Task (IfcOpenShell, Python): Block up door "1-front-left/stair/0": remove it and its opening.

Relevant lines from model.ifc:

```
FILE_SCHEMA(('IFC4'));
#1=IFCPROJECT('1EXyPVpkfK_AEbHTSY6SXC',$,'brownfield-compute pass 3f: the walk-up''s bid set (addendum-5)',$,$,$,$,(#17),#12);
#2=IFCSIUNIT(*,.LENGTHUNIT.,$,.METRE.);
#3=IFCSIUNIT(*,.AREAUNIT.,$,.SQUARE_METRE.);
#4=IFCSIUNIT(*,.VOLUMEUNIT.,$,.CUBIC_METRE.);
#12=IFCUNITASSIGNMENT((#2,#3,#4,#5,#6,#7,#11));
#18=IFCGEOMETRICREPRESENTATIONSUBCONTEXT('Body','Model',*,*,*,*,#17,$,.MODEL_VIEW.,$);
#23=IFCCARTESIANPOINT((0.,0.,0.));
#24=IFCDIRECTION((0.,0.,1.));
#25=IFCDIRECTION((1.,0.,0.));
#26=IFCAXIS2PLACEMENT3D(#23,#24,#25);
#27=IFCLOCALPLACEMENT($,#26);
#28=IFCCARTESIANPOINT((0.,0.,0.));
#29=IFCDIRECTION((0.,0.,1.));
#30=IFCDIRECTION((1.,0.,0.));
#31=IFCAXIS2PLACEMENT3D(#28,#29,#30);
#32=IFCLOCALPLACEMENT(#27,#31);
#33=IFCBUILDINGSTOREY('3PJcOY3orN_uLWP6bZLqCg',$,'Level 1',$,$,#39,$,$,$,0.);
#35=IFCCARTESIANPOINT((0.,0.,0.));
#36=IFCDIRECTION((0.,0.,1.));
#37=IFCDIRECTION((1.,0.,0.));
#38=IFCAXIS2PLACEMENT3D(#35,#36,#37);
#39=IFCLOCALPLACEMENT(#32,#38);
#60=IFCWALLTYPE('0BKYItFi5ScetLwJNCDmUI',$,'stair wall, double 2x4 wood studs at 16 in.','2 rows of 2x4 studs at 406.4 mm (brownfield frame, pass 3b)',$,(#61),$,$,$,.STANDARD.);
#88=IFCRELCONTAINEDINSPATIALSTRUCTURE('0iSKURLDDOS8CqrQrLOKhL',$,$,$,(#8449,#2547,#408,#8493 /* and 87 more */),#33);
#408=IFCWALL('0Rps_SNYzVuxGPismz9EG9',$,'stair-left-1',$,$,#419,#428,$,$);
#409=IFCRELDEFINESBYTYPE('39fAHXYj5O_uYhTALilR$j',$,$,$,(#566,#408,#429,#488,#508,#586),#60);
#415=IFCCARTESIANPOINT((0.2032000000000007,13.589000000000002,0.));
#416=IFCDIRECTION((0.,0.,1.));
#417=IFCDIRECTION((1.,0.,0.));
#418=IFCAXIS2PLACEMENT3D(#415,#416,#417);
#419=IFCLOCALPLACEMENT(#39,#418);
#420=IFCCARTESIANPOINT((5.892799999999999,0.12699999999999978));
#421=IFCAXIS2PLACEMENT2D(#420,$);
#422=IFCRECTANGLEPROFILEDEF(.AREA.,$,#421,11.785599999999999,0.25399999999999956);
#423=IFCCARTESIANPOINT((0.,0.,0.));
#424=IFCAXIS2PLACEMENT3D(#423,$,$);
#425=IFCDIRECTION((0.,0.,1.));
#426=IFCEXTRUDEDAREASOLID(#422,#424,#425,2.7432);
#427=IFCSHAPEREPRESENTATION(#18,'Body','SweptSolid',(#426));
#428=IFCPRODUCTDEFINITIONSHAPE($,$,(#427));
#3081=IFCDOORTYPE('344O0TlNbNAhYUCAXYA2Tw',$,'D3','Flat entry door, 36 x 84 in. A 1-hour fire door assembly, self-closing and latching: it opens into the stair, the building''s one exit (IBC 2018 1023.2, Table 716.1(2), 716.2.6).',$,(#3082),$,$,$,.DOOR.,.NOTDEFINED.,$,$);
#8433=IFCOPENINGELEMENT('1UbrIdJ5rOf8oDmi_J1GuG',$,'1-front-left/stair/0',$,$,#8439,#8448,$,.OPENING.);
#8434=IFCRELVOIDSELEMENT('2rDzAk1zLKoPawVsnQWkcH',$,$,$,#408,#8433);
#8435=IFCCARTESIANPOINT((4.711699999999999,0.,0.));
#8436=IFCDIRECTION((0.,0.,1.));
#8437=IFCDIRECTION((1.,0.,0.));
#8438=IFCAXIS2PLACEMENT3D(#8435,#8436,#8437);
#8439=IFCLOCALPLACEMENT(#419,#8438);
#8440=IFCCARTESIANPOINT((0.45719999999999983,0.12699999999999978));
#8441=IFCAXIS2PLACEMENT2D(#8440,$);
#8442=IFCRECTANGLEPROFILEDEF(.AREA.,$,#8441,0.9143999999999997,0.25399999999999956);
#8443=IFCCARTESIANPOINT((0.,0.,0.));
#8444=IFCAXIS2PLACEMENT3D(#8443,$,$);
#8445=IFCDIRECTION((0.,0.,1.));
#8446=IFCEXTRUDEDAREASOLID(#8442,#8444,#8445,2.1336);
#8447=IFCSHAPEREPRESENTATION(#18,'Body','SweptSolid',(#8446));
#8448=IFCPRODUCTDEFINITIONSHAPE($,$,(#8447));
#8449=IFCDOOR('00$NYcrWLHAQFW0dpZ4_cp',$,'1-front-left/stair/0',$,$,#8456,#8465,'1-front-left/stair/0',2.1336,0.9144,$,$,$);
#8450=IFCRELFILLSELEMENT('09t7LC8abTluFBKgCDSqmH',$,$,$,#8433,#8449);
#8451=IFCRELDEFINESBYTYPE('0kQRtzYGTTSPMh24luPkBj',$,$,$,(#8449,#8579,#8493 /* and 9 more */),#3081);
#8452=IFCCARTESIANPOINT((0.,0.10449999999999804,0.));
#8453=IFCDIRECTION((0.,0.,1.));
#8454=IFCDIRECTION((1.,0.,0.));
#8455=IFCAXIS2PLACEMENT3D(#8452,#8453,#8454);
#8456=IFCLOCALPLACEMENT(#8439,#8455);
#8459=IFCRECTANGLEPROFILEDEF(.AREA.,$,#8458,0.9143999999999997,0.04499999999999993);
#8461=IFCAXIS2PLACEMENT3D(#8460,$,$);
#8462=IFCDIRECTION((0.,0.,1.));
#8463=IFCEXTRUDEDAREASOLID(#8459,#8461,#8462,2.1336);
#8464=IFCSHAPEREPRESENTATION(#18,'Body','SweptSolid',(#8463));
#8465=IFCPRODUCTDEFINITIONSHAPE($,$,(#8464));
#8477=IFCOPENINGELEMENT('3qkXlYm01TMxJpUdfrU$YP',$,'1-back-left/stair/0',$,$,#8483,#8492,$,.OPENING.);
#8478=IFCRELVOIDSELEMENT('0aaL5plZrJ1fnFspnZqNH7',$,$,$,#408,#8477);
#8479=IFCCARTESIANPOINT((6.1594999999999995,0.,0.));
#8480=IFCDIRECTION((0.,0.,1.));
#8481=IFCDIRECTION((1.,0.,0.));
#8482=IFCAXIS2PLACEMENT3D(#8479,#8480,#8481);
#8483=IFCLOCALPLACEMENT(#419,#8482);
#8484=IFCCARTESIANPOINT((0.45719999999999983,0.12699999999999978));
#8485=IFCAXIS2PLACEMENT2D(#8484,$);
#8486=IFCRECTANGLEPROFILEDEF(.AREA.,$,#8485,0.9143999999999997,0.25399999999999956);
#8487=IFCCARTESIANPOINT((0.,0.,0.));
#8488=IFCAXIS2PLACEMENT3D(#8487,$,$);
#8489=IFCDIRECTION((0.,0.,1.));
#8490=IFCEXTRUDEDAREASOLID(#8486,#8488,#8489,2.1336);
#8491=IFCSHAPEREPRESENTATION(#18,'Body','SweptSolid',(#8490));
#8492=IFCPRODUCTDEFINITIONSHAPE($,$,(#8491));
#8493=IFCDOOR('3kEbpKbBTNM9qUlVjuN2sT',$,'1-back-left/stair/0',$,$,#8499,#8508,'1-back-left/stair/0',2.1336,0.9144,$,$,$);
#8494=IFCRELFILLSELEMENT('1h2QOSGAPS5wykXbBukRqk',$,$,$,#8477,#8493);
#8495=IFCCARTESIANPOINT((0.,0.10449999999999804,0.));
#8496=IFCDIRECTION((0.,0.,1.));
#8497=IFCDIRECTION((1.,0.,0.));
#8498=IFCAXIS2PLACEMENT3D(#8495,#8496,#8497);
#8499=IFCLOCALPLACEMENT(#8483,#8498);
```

```python
import ifcopenshell
import ifcopenshell.api.feature
import ifcopenshell.api.root
import ifcopenshell.geom
import ifcopenshell.util.shape

model = ifcopenshell.open("model.ifc")
settings = ifcopenshell.geom.settings()


def volume(element):
    """Net volume in cubic metres, openings subtracted."""
    shape = ifcopenshell.geom.create_shape(settings, element)
    return ifcopenshell.util.shape.get_volume(shape.geometry)


door = model.by_id(8449)
opening = door.FillsVoids[0].RelatingOpeningElement
wall = opening.VoidsElements[0].RelatingBuildingElement
before = volume(wall)

ifcopenshell.api.root.remove_product(model, product=door)
ifcopenshell.api.feature.remove_feature(model, feature=opening)

after = volume(wall)

print(f"wall volume {before:.3f} -> {after:.3f} m3")

model.write("model_edited.ifc")
```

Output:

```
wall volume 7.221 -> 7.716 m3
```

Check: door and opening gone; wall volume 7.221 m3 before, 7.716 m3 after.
